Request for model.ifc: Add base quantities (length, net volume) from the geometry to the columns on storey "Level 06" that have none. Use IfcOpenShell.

First a look at what the model holds.

```python
import ifcopenshell
import ifcopenshell.util.element
import ifcopenshell.util.unit

model = ifcopenshell.open("model.ifc")
print(model.schema)
for unit_type in ("LENGTHUNIT", "AREAUNIT", "VOLUMEUNIT"):
    print(unit_type, ifcopenshell.util.unit.calculate_unit_scale(model, unit_type))
storey = next(s for s in model.by_type("IfcBuildingStorey") if s.Name == "Level 06")
columns = [e for e in ifcopenshell.util.element.get_decomposition(storey) if e.is_a("IfcColumn")]
for e in sorted(columns, key=lambda e: e.id()):
    print(e.id(), e.is_a(), e.Name, list(ifcopenshell.util.element.get_psets(e, qtos_only=True)), sep=" | ")
```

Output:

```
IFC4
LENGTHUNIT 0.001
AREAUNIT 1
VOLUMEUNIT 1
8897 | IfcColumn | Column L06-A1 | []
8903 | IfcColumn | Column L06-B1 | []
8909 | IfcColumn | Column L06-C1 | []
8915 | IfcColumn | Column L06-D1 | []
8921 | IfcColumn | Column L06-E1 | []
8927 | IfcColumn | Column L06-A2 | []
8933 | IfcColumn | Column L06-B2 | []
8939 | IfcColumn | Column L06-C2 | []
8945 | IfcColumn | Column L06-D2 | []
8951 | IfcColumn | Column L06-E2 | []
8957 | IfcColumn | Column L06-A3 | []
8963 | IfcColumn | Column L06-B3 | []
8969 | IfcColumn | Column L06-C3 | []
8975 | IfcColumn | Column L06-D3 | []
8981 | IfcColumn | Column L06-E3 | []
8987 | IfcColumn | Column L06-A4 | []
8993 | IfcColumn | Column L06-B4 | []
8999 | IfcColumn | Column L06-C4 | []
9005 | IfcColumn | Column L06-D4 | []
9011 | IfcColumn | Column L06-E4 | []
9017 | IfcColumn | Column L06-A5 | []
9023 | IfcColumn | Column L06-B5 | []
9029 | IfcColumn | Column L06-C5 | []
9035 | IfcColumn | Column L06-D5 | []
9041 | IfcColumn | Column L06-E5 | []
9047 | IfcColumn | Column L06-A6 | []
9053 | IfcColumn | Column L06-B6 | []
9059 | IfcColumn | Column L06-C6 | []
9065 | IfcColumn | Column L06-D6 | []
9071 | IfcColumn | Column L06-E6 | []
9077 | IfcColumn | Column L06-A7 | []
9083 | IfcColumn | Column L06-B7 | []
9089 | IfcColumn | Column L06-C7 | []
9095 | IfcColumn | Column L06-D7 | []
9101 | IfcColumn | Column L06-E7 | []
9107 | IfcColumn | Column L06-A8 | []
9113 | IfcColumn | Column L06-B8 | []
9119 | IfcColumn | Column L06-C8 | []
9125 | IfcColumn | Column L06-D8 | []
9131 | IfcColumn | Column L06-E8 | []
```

```python
import ifcopenshell
import ifcopenshell.api.pset
import ifcopenshell.geom
import ifcopenshell.util.element
import ifcopenshell.util.shape
import ifcopenshell.util.unit

model = ifcopenshell.open("model.ifc")
unit_scale = ifcopenshell.util.unit.calculate_unit_scale(model)
volume_scale = ifcopenshell.util.unit.calculate_unit_scale(model, "VOLUMEUNIT")
settings = ifcopenshell.geom.settings()

storey = next(s for s in model.by_type("IfcBuildingStorey") if s.Name == "Level 06")
columns = [e for e in ifcopenshell.util.element.get_decomposition(storey) if e.is_a("IfcColumn")]

for e in sorted(columns, key=lambda e: e.id()):
    if ifcopenshell.util.element.get_psets(e, qtos_only=True, should_inherit=False):
        continue
    # Geometry comes back in metres, in the element's own axes.
    shape = ifcopenshell.geom.create_shape(settings, e)
    values = {
        "Length": ifcopenshell.util.shape.get_z(shape.geometry) / unit_scale,
        "NetVolume": ifcopenshell.util.shape.get_volume(shape.geometry) / volume_scale,
    }
    qto = ifcopenshell.api.pset.add_qto(model, product=e, name="Qto_ColumnBaseQuantities")
    ifcopenshell.api.pset.edit_qto(model, qto=qto, properties=values)
    print(e.id(), {k: round(v, 3) for k, v in values.items()})

model.write("model-out.ifc")
```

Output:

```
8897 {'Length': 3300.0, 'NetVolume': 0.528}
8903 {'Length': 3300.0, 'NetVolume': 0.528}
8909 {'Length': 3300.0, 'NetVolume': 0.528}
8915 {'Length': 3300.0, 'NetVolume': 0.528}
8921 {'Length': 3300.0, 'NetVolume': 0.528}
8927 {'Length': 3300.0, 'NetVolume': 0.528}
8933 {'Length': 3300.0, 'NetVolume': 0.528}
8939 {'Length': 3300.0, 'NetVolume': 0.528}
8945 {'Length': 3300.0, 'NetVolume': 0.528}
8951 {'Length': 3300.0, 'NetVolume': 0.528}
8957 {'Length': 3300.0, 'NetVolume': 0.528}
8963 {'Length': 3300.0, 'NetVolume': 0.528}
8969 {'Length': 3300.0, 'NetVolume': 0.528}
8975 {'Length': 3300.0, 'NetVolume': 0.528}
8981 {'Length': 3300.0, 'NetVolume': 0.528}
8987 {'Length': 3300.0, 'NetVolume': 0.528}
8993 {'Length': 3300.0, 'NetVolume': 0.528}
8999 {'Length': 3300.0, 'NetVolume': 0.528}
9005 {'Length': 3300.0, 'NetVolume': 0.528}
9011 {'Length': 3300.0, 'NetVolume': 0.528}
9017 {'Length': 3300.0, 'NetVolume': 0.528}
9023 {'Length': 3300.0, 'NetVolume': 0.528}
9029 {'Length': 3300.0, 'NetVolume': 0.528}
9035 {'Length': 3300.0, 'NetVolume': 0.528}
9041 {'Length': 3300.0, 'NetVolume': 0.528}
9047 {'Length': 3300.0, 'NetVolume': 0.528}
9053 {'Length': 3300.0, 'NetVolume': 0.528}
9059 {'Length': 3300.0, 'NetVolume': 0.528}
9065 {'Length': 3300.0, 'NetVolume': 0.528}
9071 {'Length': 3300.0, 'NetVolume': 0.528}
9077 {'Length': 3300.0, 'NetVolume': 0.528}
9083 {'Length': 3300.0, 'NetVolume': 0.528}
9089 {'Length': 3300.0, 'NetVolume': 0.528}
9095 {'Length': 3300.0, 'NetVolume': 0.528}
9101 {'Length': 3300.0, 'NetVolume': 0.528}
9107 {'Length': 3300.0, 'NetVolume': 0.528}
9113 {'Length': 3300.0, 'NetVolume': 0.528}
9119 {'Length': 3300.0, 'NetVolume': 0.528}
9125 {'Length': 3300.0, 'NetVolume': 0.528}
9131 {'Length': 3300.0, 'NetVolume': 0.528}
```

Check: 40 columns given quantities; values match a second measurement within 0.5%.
